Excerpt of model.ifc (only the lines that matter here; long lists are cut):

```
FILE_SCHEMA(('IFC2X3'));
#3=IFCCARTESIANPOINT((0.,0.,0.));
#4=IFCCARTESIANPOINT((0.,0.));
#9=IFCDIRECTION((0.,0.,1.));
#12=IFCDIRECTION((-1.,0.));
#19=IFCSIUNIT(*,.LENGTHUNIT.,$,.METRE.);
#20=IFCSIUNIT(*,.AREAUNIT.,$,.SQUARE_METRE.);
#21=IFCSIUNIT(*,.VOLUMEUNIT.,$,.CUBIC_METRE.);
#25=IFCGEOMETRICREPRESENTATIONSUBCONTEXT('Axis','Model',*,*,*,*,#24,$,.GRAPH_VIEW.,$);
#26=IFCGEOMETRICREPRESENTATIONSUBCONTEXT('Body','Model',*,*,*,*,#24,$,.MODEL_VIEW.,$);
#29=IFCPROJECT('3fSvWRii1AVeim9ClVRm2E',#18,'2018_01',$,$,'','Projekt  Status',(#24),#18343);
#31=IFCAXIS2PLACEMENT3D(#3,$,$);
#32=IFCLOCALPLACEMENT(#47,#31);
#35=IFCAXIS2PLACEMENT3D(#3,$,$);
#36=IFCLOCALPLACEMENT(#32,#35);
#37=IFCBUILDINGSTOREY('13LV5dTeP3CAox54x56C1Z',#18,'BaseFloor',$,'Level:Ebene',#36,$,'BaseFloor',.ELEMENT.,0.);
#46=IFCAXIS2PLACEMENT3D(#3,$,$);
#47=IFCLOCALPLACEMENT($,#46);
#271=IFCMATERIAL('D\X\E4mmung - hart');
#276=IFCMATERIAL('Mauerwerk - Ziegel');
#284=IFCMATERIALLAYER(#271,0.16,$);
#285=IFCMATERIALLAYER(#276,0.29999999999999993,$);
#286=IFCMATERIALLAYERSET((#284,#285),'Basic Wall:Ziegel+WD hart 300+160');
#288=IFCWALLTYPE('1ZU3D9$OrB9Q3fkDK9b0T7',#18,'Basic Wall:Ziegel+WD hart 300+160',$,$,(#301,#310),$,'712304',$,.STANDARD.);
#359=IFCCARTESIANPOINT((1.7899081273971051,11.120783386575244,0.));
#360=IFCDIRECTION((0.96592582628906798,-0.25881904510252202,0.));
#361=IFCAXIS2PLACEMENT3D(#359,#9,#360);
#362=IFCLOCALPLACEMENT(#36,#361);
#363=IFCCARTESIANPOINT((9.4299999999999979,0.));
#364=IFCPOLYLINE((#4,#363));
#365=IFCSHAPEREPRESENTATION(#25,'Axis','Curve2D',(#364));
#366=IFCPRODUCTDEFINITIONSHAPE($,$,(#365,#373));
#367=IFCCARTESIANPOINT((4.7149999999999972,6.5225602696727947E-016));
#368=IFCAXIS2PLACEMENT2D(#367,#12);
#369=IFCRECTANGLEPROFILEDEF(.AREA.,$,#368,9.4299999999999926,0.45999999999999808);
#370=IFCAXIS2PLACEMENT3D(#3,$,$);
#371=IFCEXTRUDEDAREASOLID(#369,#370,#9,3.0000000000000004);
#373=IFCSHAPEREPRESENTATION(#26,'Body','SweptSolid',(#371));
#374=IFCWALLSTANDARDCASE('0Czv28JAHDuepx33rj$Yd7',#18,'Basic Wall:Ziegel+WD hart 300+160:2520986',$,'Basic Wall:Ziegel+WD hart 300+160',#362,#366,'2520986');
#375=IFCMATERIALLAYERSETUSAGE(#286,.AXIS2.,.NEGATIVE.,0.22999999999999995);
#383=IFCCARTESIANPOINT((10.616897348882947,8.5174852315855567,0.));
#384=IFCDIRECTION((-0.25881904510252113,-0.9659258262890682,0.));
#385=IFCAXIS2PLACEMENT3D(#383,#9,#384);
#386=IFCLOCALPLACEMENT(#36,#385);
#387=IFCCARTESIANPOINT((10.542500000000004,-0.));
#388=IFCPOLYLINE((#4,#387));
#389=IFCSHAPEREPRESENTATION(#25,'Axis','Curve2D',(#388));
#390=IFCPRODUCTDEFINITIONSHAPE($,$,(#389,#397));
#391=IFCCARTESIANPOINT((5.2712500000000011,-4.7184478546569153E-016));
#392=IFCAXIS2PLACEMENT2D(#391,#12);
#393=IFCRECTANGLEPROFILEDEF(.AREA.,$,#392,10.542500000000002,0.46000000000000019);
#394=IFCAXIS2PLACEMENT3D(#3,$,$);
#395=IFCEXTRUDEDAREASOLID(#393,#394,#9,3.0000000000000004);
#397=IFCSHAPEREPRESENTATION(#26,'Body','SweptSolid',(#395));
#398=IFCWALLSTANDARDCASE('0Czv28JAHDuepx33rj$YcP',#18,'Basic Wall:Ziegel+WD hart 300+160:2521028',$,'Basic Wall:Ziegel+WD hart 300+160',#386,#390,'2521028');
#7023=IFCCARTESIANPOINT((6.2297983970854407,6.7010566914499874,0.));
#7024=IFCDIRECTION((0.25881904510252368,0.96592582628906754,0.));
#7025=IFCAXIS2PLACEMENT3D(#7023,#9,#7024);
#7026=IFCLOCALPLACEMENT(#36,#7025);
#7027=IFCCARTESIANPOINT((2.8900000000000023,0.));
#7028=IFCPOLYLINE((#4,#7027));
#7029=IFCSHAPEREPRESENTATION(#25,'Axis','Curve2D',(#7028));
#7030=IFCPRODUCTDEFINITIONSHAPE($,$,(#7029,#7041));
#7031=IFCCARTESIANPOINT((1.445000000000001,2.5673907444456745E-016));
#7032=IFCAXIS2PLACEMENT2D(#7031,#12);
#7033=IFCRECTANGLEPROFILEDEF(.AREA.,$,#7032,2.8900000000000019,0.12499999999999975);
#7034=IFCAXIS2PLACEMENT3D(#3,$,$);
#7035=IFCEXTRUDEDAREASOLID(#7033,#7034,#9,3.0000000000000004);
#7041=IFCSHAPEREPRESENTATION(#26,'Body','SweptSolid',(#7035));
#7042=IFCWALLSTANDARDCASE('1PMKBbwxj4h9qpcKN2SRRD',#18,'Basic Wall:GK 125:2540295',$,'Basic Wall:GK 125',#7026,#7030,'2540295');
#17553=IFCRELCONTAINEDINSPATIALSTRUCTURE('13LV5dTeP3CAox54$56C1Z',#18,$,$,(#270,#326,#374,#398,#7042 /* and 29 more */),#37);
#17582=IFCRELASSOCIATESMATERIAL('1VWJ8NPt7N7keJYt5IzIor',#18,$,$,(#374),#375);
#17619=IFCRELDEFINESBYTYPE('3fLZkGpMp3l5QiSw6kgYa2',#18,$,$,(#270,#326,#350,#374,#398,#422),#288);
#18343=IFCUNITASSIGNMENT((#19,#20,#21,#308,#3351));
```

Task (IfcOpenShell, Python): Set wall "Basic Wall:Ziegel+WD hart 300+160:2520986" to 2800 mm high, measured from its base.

```python
import ifcopenshell
import ifcopenshell.geom
import ifcopenshell.util.representation
import ifcopenshell.util.shape

model = ifcopenshell.open("model.ifc")
settings = ifcopenshell.geom.settings()


def volume(element):
    """Net volume in cubic metres, openings subtracted."""
    shape = ifcopenshell.geom.create_shape(settings, element)
    return ifcopenshell.util.shape.get_volume(shape.geometry)


wall = model.by_id(374)
before = volume(wall)

body = ifcopenshell.util.representation.get_representation(wall, "Model", "Body")
solid = body.Items[0]
old_height = solid.Depth
solid.Depth = 2.8
after = volume(wall)

print(f"height {old_height:g} -> {solid.Depth:g}, volume {before:.3f} -> {after:.3f} m3")

model.write("model_edited.ifc")
```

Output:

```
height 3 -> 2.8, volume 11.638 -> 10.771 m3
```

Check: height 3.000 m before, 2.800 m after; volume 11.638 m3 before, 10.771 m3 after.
